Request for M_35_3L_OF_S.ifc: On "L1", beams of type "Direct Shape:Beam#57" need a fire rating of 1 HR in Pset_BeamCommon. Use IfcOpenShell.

First a look at what the model holds.

```python
import ifcopenshell
import ifcopenshell.util.element

model = ifcopenshell.open("M_35_3L_OF_S.ifc")
print(model.schema)
storey = next(s for s in model.by_type("IfcBuildingStorey") if s.Name == "L1")
beams = [e for e in ifcopenshell.util.element.get_decomposition(storey) if e.is_a("IfcBeam")]
seen = {}
for e in beams:
    element_type = ifcopenshell.util.element.get_type(e)
    key = (element_type.Name if element_type != e and element_type else None, ifcopenshell.util.element.get_pset(e, "Pset_BeamCommon", "FireRating"))
    seen[key] = seen.get(key, 0) + 1
for (name, value), count in sorted(seen.items(), key=str):
    print(count, "x", name, "|", value)
```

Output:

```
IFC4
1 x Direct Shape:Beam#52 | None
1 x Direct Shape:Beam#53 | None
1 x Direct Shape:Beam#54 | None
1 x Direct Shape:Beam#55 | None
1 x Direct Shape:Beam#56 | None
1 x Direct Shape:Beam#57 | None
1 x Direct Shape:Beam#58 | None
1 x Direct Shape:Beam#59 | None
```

```python
import ifcopenshell
import ifcopenshell.api.pset
import ifcopenshell.util.element

model = ifcopenshell.open("M_35_3L_OF_S.ifc")

storey = next(s for s in model.by_type("IfcBuildingStorey") if s.Name == "L1")
beams = [e for e in ifcopenshell.util.element.get_decomposition(storey) if e.is_a("IfcBeam")]

count = 0
for e in beams:
    element_type = ifcopenshell.util.element.get_type(e)
    if element_type in (None, e) or element_type.Name != "Direct Shape:Beam#57":
        continue
    # add_pset returns the element's existing set when there is one.
    pset = ifcopenshell.api.pset.add_pset(model, product=e, name="Pset_BeamCommon")
    ifcopenshell.api.pset.edit_pset(model, pset=pset, properties={"FireRating": "1 HR"})
    count += 1

print(count, "beams updated")

model.write("M_35_3L_OF_S_v2.ifc")
```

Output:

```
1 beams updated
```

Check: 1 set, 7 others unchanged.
